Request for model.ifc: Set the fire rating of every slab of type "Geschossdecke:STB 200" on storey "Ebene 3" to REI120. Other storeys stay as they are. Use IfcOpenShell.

First a look at what the model holds.

```python
import ifcopenshell
import ifcopenshell.util.element

model = ifcopenshell.open("model.ifc")
print(model.schema)
storey = next(s for s in model.by_type("IfcBuildingStorey") if s.Name == "Ebene 3")
slabs = [e for e in ifcopenshell.util.element.get_decomposition(storey) if e.is_a("IfcSlab")]
seen = {}
for e in slabs:
    element_type = ifcopenshell.util.element.get_type(e)
    key = (element_type.Name if element_type != e and element_type else None, ifcopenshell.util.element.get_pset(e, "Pset_SlabCommon", "FireRating"))
    seen[key] = seen.get(key, 0) + 1
for (name, value), count in sorted(seen.items(), key=str):
    print(count, "x", name, "|", value)
```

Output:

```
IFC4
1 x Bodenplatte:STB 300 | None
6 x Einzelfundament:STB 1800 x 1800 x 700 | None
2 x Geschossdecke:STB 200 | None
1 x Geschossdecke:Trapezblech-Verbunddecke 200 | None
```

```python
import ifcopenshell
import ifcopenshell.api.pset
import ifcopenshell.util.element

model = ifcopenshell.open("model.ifc")

storey = next(s for s in model.by_type("IfcBuildingStorey") if s.Name == "Ebene 3")
slabs = [e for e in ifcopenshell.util.element.get_decomposition(storey) if e.is_a("IfcSlab")]

count = 0
for e in slabs:
    element_type = ifcopenshell.util.element.get_type(e)
    if element_type in (None, e) or element_type.Name != "Geschossdecke:STB 200":
        continue
    # add_pset returns the element's existing set when there is one.
    pset = ifcopenshell.api.pset.add_pset(model, product=e, name="Pset_SlabCommon")
    ifcopenshell.api.pset.edit_pset(model, pset=pset, properties={"FireRating": "REI120"})
    count += 1

print(count, "slabs updated")

model.write("model_rev.ifc")
```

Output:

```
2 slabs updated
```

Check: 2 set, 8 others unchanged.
